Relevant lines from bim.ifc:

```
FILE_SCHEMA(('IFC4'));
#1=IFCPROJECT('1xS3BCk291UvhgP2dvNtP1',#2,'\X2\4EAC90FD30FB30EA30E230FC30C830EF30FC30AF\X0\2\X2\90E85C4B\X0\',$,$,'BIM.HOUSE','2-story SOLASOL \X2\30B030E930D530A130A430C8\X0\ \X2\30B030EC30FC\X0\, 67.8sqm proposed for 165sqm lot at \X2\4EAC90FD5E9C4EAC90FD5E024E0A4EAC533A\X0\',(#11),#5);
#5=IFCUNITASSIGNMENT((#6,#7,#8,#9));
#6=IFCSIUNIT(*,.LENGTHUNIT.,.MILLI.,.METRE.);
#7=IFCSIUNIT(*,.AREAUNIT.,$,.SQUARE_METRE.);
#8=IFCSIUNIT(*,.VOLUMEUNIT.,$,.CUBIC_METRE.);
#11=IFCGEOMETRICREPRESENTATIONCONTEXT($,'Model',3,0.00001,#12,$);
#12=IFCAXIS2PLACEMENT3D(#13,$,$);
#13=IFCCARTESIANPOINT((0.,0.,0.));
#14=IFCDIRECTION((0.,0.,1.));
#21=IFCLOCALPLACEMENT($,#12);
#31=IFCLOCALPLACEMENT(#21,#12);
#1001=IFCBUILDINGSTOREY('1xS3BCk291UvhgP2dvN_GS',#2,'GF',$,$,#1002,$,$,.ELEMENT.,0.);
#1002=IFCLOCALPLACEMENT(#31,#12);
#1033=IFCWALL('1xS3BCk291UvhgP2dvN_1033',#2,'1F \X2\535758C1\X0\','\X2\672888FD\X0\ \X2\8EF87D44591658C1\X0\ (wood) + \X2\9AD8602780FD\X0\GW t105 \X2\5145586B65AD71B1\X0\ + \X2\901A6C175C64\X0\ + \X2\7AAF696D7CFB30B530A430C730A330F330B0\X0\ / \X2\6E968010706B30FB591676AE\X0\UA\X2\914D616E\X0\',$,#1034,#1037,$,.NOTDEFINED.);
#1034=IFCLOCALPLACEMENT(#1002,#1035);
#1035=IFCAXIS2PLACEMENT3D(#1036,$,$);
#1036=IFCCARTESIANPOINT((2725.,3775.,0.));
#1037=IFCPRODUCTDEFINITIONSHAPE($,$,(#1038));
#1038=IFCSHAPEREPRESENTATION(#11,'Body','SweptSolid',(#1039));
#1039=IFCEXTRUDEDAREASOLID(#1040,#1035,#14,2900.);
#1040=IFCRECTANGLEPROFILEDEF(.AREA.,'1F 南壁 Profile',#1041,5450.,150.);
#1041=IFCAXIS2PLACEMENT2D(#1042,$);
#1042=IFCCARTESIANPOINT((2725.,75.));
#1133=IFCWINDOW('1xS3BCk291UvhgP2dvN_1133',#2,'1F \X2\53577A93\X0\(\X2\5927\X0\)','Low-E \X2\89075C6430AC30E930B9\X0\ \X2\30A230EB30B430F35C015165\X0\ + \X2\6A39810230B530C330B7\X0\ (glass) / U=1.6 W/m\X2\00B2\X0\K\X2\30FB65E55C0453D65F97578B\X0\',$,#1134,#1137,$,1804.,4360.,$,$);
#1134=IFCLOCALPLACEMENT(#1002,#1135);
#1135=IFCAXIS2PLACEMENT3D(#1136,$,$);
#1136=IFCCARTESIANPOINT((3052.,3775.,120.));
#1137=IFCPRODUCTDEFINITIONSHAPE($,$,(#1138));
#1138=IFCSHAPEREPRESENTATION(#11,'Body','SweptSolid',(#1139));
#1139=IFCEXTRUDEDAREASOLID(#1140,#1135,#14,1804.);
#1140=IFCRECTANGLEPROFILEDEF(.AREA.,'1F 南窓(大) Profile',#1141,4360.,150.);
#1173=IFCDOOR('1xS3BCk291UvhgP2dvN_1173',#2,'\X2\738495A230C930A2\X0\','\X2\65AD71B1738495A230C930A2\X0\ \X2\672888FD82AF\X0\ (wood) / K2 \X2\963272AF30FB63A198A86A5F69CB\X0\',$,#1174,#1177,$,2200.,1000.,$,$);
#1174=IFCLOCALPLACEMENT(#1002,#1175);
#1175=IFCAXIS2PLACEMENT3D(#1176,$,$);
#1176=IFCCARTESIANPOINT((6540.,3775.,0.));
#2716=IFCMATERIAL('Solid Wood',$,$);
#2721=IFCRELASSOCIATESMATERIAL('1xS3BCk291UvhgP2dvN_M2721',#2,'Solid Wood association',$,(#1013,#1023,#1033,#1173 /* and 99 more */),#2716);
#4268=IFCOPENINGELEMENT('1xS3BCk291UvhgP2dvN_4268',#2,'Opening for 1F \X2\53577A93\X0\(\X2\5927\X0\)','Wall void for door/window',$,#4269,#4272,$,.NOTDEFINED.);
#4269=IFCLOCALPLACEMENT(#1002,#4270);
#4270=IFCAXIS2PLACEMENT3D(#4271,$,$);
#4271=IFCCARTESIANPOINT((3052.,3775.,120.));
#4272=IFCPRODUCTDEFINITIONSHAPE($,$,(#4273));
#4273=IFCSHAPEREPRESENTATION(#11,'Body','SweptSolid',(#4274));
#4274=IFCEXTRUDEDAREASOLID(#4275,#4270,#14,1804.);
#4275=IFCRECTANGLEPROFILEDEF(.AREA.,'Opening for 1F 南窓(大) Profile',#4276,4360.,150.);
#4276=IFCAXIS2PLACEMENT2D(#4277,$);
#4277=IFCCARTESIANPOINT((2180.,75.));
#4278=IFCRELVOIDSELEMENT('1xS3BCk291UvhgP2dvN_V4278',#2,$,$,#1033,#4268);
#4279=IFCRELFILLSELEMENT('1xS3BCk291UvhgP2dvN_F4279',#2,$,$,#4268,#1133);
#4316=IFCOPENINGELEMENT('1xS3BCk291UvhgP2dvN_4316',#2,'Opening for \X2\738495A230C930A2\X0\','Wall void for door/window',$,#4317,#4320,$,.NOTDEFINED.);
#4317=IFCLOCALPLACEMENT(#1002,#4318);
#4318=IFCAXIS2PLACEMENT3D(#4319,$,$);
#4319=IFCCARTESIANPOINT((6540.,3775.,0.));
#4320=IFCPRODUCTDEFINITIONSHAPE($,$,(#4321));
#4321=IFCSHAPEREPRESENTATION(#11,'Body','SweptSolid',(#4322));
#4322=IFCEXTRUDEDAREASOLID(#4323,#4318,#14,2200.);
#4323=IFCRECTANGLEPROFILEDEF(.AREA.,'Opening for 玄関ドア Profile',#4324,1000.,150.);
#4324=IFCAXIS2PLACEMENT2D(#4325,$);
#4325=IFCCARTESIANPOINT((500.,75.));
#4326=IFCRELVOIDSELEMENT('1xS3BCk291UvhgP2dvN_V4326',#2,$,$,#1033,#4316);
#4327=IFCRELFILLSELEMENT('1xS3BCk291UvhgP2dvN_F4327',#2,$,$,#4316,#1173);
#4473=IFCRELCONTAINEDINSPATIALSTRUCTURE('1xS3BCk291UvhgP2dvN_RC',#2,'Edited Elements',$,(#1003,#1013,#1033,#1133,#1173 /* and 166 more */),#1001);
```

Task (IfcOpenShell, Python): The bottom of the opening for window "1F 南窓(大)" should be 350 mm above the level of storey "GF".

```python
import numpy as np
import ifcopenshell
import ifcopenshell.api.geometry
import ifcopenshell.geom
import ifcopenshell.util.element
import ifcopenshell.util.placement
import ifcopenshell.util.shape
import ifcopenshell.util.unit

model = ifcopenshell.open("bim.ifc")
unit_scale = ifcopenshell.util.unit.calculate_unit_scale(model)

window = model.by_guid("1xS3BCk291UvhgP2dvN_1133")
opening = window.FillsVoids[0].RelatingOpeningElement
storey = ifcopenshell.util.element.get_container(window, ifc_class="IfcBuildingStorey")
level = ifcopenshell.util.placement.get_local_placement(storey.ObjectPlacement)[2, 3]

# The opening's origin need not be at the sill, so measure its lowest point.
shape = ifcopenshell.geom.create_shape(ifcopenshell.geom.settings(), opening)
bottom = ifcopenshell.util.shape.get_shape_bottom_elevation(shape, shape.geometry) / unit_scale
dz = level + 0.35 / unit_scale - bottom

shift = np.array([0.0, 0.0, dz])
# The window is not placed relative to its opening, so move both.
for product in (opening, window):
    matrix = ifcopenshell.util.placement.get_local_placement(product.ObjectPlacement)
    matrix[:3, 3] += shift
    ifcopenshell.api.geometry.edit_object_placement(model, product=product, matrix=matrix, is_si=False)

print(f"moved by {dz * unit_scale:+.3f} m")

model.write("bim-out.ifc")
```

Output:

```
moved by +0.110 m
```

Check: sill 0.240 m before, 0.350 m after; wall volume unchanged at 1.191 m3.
